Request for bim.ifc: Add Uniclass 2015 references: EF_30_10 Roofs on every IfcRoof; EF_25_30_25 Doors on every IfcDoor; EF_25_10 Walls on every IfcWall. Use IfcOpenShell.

First a look at what the model holds.

```python
import ifcopenshell

model = ifcopenshell.open("bim.ifc")
print(model.schema)
print("classifications:", [c.Name for c in model.by_type("IfcClassification")])
for ifc_class in ("IfcDoor", "IfcRoof", "IfcStair", "IfcWall", "IfcWindow"):
    print(ifc_class, len(model.by_type(ifc_class)))
```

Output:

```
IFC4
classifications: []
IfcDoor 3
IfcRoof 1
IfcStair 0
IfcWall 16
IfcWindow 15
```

```python
import ifcopenshell
import ifcopenshell.api.classification

model = ifcopenshell.open("bim.ifc")

system = ifcopenshell.api.classification.add_classification(model, classification="Uniclass 2015")

codes = {
    "IfcRoof": ("EF_30_10", "Roofs"),
    "IfcDoor": ("EF_25_30_25", "Doors"),
    "IfcWall": ("EF_25_10", "Walls"),
}
for ifc_class, (code, name) in codes.items():
    products = model.by_type(ifc_class)
    ifcopenshell.api.classification.add_reference(
        model, products=products, classification=system, identification=code, name=name
    )
    print(code, len(products))

model.write("bim_rev.ifc")
```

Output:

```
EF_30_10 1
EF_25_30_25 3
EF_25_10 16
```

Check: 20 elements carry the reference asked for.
